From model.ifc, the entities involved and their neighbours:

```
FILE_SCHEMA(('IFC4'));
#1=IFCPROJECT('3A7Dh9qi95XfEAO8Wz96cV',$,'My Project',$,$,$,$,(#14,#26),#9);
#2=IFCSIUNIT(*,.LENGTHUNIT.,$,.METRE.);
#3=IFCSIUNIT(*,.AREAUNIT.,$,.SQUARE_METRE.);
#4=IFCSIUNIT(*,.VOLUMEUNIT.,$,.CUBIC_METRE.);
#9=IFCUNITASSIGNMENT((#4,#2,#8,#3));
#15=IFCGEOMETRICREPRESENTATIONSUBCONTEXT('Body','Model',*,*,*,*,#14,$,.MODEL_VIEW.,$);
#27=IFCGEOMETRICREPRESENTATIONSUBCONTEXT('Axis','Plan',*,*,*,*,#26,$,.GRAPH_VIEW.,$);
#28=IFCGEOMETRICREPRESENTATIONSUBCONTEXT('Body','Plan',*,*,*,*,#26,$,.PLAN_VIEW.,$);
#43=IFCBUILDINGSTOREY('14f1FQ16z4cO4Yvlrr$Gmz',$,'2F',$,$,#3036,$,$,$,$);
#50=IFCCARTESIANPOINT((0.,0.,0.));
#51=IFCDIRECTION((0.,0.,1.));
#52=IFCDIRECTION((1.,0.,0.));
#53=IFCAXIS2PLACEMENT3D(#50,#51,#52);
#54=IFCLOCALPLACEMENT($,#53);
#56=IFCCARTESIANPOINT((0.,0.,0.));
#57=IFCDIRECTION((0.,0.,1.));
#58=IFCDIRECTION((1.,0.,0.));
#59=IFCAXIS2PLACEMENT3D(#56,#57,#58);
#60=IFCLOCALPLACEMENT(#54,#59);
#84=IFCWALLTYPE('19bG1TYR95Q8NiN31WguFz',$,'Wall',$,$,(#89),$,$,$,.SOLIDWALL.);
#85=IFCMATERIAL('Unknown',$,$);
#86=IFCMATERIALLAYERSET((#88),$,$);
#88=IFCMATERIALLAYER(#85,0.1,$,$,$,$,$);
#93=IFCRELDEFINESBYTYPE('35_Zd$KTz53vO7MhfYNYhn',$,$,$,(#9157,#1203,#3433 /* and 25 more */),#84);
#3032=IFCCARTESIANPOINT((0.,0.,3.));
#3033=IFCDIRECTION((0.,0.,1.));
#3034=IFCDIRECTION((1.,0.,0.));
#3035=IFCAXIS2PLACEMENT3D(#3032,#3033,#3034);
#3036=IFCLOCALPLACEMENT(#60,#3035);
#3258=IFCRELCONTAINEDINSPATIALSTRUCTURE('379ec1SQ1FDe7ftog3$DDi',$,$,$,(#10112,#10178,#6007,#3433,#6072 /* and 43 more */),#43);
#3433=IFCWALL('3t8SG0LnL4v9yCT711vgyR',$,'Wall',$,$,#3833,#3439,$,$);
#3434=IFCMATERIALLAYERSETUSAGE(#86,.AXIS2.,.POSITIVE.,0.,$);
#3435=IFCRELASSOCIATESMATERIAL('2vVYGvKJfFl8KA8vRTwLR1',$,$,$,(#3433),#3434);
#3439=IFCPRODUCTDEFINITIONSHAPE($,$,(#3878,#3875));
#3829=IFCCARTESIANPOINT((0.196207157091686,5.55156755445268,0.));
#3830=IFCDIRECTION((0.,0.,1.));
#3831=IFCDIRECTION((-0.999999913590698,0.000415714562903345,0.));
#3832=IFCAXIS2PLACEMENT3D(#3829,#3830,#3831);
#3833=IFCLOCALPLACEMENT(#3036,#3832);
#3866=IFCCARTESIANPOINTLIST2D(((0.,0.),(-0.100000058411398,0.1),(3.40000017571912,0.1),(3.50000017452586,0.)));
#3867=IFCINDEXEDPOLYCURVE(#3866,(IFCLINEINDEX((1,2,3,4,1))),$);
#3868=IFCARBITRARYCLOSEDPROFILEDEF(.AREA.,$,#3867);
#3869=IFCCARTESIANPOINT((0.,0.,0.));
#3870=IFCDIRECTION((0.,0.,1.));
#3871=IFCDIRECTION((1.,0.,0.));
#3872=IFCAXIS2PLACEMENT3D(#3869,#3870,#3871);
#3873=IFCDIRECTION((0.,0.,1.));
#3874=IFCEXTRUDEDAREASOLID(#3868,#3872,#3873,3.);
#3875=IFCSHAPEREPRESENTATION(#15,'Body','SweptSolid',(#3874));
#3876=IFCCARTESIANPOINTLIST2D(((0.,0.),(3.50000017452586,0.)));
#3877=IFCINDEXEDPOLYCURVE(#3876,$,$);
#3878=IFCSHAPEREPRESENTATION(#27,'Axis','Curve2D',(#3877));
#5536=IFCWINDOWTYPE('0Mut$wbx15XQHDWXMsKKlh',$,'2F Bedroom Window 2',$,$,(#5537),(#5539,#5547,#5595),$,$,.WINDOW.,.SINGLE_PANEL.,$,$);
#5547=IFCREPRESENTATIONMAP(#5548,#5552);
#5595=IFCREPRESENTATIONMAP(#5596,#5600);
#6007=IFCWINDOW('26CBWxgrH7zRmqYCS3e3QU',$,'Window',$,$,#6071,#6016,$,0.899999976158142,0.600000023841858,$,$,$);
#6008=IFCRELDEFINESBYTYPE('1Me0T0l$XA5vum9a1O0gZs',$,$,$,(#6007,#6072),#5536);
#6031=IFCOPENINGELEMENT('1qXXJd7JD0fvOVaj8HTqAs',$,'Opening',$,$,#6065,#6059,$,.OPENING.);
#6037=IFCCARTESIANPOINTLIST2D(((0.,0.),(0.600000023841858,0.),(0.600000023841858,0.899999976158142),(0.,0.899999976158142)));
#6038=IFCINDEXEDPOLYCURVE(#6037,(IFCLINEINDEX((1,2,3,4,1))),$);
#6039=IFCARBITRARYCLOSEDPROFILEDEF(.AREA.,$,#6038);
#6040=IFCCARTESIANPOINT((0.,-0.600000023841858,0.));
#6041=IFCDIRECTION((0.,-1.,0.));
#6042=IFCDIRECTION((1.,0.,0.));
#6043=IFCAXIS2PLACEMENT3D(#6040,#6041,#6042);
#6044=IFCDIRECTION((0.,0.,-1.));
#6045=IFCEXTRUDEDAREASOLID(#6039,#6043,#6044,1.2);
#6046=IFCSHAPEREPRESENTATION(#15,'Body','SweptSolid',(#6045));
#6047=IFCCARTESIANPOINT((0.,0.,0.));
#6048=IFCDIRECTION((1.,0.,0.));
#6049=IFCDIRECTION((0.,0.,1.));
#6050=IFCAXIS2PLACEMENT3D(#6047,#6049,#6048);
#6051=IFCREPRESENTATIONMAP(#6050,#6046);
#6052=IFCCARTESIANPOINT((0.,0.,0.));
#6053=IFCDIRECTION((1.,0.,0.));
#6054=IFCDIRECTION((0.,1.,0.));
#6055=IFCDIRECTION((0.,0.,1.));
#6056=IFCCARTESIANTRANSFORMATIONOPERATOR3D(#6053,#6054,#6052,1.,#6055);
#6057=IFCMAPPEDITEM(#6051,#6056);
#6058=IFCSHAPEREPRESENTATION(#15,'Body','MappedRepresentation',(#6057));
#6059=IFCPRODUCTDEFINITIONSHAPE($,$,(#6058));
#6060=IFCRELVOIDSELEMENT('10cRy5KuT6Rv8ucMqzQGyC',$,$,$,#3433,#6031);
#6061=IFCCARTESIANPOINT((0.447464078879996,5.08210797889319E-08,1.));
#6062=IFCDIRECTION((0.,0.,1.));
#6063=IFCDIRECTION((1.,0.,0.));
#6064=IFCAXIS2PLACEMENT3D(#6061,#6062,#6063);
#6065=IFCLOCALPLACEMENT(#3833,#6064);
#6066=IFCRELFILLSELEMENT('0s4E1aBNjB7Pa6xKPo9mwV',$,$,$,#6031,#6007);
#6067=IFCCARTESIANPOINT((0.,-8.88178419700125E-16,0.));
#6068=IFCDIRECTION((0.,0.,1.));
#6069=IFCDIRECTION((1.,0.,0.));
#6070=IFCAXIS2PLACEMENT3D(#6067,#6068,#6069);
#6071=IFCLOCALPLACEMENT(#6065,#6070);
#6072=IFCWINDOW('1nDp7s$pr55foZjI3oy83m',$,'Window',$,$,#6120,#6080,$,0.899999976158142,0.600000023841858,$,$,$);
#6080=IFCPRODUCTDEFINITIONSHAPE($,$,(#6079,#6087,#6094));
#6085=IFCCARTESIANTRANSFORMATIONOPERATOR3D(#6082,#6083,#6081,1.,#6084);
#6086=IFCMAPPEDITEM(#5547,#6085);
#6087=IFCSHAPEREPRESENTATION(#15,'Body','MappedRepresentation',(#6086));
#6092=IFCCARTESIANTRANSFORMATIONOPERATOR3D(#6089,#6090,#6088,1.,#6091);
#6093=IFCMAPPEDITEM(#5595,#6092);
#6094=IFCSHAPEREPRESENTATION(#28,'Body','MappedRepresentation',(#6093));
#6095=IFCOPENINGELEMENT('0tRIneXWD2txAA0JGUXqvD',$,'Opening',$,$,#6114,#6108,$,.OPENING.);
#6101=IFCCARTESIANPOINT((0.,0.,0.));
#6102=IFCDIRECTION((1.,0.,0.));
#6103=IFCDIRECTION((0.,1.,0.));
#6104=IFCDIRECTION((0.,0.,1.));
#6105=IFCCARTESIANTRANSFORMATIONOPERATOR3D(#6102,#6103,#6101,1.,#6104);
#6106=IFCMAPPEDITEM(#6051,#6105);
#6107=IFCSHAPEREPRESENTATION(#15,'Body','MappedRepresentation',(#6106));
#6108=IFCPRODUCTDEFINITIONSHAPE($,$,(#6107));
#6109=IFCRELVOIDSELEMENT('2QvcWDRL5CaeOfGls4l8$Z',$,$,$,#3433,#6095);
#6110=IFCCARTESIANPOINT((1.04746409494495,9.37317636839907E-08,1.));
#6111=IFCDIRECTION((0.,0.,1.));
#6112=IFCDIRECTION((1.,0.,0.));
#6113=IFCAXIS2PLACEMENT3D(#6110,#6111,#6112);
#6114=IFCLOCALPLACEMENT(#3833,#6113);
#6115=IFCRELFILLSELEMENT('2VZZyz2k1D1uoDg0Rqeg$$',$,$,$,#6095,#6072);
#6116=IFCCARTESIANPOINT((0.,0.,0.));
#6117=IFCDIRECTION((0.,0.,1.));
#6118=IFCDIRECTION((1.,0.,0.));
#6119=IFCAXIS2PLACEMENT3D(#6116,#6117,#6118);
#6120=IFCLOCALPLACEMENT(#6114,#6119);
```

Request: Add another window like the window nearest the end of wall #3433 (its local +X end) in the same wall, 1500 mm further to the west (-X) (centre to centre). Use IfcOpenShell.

```python
import ifcopenshell
import ifcopenshell.api.feature
import ifcopenshell.api.geometry
import ifcopenshell.api.root
import ifcopenshell.geom
import ifcopenshell.util.element
import ifcopenshell.util.placement
import ifcopenshell.util.shape

model = ifcopenshell.open("model.ifc")
settings = ifcopenshell.geom.settings()


def volume(element):
    """Net volume in cubic metres, openings subtracted."""
    shape = ifcopenshell.geom.create_shape(settings, element)
    return ifcopenshell.util.shape.get_volume(shape.geometry)


window = model.by_guid("1nDp7s$pr55foZjI3oy83m")
opening = window.FillsVoids[0].RelatingOpeningElement
wall = opening.VoidsElements[0].RelatingBuildingElement
before = volume(wall)
shift = ifcopenshell.util.placement.get_local_placement(wall.ObjectPlacement)[:3, 0] * 1.5

# copy_class copies the void relationship, type, container and properties, but no geometry.
new_opening = ifcopenshell.api.root.copy_class(model, product=opening)
new_opening.Representation = ifcopenshell.util.element.copy_deep(
    model, opening.Representation, exclude=["IfcGeometricRepresentationContext", "IfcRepresentationMap"]
)
new_window = ifcopenshell.api.root.copy_class(model, product=window)
new_window.Representation = ifcopenshell.util.element.copy_deep(
    model, window.Representation, exclude=["IfcGeometricRepresentationContext", "IfcRepresentationMap"]
)
ifcopenshell.api.feature.add_filling(model, opening=new_opening, element=new_window)

for old, new in ((opening, new_opening), (window, new_window)):
    matrix = ifcopenshell.util.placement.get_local_placement(old.ObjectPlacement)
    matrix[:3, 3] += shift
    ifcopenshell.api.geometry.edit_object_placement(model, product=new, matrix=matrix, is_si=False)

after = volume(wall)

print(f"wall volume {before:.3f} -> {after:.3f} m3")

model.write("model-out.ifc")
```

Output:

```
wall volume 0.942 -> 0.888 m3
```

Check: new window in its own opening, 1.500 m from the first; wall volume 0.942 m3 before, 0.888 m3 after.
